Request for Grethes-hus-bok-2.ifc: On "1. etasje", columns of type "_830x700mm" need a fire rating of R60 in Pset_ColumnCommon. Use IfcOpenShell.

First a look at what the model holds.

```python
import ifcopenshell
import ifcopenshell.util.element

model = ifcopenshell.open("Grethes-hus-bok-2.ifc")
print(model.schema)
storey = next(s for s in model.by_type("IfcBuildingStorey") if s.Name == "1. etasje")
columns = [e for e in ifcopenshell.util.element.get_decomposition(storey) if e.is_a("IfcColumn")]
seen = {}
for e in columns:
    element_type = ifcopenshell.util.element.get_type(e)
    key = (element_type.Name if element_type != e and element_type else None, ifcopenshell.util.element.get_pset(e, "Pset_ColumnCommon", "FireRating"))
    seen[key] = seen.get(key, 0) + 1
for (name, value), count in sorted(seen.items(), key=str):
    print(count, "x", name, "|", value)
```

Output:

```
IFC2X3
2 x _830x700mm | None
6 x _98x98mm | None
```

```python
import ifcopenshell
import ifcopenshell.api.pset
import ifcopenshell.util.element

model = ifcopenshell.open("Grethes-hus-bok-2.ifc")

storey = next(s for s in model.by_type("IfcBuildingStorey") if s.Name == "1. etasje")
columns = [e for e in ifcopenshell.util.element.get_decomposition(storey) if e.is_a("IfcColumn")]

count = 0
for e in columns:
    element_type = ifcopenshell.util.element.get_type(e)
    if element_type in (None, e) or element_type.Name != "_830x700mm":
        continue
    # add_pset returns the element's existing set when there is one.
    pset = ifcopenshell.api.pset.add_pset(model, product=e, name="Pset_ColumnCommon")
    ifcopenshell.api.pset.edit_pset(model, pset=pset, properties={"FireRating": "R60"})
    count += 1

print(count, "columns updated")

model.write("Grethes-hus-bok-2_edited.ifc")
```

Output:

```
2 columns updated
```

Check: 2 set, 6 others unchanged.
